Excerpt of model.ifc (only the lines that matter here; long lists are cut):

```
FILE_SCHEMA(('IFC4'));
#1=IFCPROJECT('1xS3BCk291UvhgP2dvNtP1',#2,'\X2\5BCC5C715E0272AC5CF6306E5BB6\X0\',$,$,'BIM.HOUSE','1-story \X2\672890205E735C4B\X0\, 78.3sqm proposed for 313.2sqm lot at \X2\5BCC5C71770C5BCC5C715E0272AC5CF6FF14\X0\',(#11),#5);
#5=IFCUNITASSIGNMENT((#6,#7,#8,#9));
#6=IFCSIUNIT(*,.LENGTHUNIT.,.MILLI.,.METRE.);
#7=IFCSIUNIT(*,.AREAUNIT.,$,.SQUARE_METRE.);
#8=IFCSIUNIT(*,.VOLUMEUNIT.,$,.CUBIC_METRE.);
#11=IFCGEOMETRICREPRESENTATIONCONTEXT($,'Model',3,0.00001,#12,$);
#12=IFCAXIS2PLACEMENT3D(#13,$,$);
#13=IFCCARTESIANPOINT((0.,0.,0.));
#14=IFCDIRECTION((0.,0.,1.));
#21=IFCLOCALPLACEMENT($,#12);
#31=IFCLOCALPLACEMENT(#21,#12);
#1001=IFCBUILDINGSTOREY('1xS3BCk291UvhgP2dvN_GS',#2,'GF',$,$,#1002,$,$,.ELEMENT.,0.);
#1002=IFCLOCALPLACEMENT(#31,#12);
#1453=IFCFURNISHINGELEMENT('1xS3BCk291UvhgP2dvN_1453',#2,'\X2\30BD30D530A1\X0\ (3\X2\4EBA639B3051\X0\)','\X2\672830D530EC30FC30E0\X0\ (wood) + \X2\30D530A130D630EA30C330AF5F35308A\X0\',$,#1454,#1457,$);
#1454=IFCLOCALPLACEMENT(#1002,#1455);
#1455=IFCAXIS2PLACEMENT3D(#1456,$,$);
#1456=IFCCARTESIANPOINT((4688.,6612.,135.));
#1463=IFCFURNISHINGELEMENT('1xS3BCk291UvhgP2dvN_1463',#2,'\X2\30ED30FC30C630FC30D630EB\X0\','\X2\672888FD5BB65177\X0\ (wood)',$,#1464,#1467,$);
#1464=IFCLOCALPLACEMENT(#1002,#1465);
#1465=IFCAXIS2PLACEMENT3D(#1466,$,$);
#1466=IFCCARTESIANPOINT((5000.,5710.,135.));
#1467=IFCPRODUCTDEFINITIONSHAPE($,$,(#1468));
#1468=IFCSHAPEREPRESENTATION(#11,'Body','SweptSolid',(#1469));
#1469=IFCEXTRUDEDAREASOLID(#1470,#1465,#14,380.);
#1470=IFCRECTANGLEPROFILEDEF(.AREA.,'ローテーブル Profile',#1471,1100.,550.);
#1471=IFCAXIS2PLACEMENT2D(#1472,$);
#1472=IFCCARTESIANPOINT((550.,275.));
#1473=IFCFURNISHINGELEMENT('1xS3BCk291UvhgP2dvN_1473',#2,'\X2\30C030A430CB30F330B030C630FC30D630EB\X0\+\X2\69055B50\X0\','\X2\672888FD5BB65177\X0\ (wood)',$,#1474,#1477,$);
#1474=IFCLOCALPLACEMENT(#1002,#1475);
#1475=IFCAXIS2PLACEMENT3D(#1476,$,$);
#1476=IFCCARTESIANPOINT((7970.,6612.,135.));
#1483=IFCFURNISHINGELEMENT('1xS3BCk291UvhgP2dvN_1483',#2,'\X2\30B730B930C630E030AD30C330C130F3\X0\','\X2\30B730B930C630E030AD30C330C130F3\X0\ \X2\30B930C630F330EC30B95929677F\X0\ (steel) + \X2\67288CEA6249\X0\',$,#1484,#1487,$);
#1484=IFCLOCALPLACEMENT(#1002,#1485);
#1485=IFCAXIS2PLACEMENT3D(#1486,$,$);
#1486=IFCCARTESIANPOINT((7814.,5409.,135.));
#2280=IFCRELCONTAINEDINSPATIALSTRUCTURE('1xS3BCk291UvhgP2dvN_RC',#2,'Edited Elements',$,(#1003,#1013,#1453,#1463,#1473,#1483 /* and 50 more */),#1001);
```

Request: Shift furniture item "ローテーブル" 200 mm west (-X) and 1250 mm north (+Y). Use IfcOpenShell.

```python
import ifcopenshell
import ifcopenshell.api.geometry
import ifcopenshell.util.placement
import ifcopenshell.util.unit

model = ifcopenshell.open("model.ifc")
unit_scale = ifcopenshell.util.unit.calculate_unit_scale(model)

item = model.by_guid("1xS3BCk291UvhgP2dvN_1463")
matrix = ifcopenshell.util.placement.get_local_placement(item.ObjectPlacement)
matrix[0, 3] -= 0.2 / unit_scale
matrix[1, 3] += 1.25 / unit_scale
ifcopenshell.api.geometry.edit_object_placement(model, product=item, matrix=matrix, is_si=False)

print(ifcopenshell.util.placement.get_local_placement(item.ObjectPlacement).round(3) + 0.0)

model.write("model-out.ifc")
```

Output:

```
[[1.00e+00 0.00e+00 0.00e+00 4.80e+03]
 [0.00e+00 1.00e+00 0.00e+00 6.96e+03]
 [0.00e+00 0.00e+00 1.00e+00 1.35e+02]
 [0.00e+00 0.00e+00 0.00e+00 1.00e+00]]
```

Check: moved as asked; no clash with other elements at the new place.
